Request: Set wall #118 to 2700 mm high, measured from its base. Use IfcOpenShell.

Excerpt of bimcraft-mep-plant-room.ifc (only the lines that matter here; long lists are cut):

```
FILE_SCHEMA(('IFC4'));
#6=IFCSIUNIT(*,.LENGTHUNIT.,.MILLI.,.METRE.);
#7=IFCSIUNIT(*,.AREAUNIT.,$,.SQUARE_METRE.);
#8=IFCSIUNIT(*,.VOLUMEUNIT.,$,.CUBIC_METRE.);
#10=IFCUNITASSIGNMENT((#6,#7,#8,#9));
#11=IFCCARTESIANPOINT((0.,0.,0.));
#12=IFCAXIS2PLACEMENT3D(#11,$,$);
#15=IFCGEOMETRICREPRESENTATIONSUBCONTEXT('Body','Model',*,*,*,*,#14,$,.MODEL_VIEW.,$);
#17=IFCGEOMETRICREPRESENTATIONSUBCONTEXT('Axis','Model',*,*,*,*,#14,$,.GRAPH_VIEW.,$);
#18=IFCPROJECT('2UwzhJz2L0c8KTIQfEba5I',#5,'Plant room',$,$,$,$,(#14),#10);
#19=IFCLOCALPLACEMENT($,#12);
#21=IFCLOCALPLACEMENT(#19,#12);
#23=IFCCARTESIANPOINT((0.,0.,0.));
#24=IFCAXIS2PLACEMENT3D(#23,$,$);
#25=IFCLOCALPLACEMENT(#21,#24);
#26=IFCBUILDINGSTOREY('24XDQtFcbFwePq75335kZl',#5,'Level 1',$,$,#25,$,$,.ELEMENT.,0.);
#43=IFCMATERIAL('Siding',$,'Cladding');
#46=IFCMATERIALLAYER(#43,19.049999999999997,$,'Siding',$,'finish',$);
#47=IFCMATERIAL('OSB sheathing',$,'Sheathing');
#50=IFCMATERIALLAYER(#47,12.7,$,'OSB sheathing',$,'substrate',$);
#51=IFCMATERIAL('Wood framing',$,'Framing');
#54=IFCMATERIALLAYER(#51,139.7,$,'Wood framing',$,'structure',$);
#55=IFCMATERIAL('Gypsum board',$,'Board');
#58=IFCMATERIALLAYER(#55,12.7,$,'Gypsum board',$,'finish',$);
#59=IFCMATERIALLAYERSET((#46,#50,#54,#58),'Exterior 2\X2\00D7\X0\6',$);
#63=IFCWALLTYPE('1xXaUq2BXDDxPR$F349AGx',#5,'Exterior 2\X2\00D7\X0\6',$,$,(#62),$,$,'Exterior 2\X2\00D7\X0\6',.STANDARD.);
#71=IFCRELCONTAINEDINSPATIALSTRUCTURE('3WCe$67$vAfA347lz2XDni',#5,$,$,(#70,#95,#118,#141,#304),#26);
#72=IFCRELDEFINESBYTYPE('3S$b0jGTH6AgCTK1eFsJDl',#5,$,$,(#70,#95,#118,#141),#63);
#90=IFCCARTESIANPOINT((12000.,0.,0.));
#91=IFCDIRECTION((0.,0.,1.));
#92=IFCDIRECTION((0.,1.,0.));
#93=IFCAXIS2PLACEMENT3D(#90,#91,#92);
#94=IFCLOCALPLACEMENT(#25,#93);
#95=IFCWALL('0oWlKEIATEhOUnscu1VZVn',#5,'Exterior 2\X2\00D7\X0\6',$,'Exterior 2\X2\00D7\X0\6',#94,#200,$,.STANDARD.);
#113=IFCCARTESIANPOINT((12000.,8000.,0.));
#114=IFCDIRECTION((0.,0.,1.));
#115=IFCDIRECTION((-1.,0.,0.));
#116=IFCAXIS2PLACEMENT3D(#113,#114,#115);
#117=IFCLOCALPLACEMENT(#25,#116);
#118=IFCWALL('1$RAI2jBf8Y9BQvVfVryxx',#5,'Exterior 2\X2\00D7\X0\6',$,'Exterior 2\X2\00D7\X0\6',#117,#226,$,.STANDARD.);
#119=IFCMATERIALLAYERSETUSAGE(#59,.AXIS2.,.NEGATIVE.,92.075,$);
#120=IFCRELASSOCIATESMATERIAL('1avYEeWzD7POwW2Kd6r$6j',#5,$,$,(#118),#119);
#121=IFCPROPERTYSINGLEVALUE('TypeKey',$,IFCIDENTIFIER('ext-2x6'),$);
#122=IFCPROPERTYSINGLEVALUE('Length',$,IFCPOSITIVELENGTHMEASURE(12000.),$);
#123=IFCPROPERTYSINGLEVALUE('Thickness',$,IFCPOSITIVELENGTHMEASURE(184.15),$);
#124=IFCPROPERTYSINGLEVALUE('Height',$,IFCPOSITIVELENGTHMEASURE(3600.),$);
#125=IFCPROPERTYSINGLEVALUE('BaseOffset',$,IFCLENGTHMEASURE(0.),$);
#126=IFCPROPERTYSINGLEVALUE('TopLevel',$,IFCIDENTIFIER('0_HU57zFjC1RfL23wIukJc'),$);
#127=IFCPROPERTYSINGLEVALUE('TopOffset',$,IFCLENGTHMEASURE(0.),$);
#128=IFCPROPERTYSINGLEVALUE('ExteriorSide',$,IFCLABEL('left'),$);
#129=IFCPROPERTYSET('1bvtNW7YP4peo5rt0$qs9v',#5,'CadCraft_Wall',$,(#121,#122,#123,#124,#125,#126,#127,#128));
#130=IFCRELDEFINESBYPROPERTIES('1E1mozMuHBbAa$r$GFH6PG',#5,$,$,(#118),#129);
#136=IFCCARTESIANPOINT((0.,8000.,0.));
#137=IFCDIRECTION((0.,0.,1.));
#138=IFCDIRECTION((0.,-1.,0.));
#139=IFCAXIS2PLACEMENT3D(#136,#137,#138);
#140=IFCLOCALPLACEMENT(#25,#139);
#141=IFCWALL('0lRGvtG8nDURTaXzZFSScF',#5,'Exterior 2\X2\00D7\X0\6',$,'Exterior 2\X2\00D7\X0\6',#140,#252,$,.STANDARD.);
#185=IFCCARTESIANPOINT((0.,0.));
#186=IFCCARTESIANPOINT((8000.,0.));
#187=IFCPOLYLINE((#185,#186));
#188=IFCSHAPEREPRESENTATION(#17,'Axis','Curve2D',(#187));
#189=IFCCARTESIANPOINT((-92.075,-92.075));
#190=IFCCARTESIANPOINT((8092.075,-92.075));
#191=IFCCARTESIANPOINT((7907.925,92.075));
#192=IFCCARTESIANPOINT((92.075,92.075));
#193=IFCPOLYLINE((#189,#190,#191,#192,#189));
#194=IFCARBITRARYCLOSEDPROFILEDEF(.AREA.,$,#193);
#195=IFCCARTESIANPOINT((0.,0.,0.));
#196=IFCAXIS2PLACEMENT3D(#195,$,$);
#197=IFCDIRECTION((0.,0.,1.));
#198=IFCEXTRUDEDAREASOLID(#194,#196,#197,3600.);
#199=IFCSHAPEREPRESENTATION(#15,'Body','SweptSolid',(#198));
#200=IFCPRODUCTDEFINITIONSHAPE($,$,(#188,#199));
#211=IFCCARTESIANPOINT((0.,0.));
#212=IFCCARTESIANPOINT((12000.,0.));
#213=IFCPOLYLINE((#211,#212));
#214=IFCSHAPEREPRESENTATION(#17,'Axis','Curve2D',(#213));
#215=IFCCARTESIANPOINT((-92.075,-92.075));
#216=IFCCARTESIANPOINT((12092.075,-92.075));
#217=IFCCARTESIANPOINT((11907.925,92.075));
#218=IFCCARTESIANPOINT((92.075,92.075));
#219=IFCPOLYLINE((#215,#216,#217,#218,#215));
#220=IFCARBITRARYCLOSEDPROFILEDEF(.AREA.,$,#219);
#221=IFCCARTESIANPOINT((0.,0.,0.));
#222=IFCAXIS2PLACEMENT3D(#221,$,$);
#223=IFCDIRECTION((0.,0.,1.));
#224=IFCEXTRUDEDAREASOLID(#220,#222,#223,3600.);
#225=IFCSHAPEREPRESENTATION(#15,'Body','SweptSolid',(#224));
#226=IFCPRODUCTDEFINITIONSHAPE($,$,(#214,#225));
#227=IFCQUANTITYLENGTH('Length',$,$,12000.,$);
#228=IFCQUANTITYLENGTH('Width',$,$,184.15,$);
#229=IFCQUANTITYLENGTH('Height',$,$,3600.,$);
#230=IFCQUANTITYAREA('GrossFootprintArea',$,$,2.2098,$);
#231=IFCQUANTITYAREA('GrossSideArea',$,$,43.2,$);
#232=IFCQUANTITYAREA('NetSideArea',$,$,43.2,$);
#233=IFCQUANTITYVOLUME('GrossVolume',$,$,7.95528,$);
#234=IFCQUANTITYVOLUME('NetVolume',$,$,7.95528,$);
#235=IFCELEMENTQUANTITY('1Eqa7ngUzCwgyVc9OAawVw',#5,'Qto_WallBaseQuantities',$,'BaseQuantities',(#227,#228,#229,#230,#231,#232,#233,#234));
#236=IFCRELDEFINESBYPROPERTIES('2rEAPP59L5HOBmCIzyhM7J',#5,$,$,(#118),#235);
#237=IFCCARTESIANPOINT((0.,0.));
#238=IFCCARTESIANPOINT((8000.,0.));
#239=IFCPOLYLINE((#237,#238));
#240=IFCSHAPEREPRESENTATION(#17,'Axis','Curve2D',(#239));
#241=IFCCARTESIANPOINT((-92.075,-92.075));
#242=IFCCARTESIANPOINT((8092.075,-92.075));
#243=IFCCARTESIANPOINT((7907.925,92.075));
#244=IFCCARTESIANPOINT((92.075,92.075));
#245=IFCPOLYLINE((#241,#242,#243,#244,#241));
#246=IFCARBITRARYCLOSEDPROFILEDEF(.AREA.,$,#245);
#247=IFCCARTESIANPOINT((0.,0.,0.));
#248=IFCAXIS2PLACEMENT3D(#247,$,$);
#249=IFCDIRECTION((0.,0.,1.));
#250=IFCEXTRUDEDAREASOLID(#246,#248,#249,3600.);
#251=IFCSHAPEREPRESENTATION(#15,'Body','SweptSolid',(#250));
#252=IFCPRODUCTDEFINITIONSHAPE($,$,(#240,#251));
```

```python
import ifcopenshell
import ifcopenshell.api.pset
import ifcopenshell.geom
import ifcopenshell.util.element
import ifcopenshell.util.representation
import ifcopenshell.util.shape
import ifcopenshell.util.unit

model = ifcopenshell.open("bimcraft-mep-plant-room.ifc")
unit_scale = ifcopenshell.util.unit.calculate_unit_scale(model)
area_scale = ifcopenshell.util.unit.calculate_unit_scale(model, "AREAUNIT")
volume_scale = ifcopenshell.util.unit.calculate_unit_scale(model, "VOLUMEUNIT")
settings = ifcopenshell.geom.settings()


def volume(element):
    """Net volume in cubic metres, openings subtracted."""
    shape = ifcopenshell.geom.create_shape(settings, element)
    return ifcopenshell.util.shape.get_volume(shape.geometry)


wall = model.by_guid("1$RAI2jBf8Y9BQvVfVryxx")
before = volume(wall)

body = ifcopenshell.util.representation.get_representation(wall, "Model", "Body")
solid = body.Items[0]
old_height = solid.Depth
solid.Depth = 2700.0
after = volume(wall)
thickness = 0.1841  # wall thickness in metres

# Update the stored height, areas and volumes.
pset = model.by_id(ifcopenshell.util.element.get_pset(wall, "CadCraft_Wall", should_inherit=False)["id"])
ifcopenshell.api.pset.edit_pset(model, pset=pset, properties={
    "Height": model.create_entity("IfcPositiveLengthMeasure", solid.Depth),
})
qto = model.by_id(ifcopenshell.util.element.get_pset(wall, "Qto_WallBaseQuantities", should_inherit=False)["id"])
ifcopenshell.api.pset.edit_qto(model, qto=qto, properties={
    "Height": solid.Depth,
    "GrossSideArea": ifcopenshell.util.element.get_pset(wall, "Qto_WallBaseQuantities", "GrossSideArea") * solid.Depth / old_height,
    "NetSideArea": after / thickness / area_scale,
    "GrossVolume": ifcopenshell.util.element.get_pset(wall, "Qto_WallBaseQuantities", "GrossVolume") * solid.Depth / old_height,
    "NetVolume": after / volume_scale,
})

print(f"height {old_height:g} -> {solid.Depth:g}, volume {before:.3f} -> {after:.3f} m3")

model.write("bimcraft-mep-plant-room_updated.ifc")
```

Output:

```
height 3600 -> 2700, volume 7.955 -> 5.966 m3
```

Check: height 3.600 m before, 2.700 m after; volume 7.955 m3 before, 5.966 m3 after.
